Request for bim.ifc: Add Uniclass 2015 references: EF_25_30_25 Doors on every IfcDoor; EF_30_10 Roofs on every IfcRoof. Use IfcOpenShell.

First a look at what the model holds.

```python
import ifcopenshell

model = ifcopenshell.open("bim.ifc")
print(model.schema)
print("classifications:", [c.Name for c in model.by_type("IfcClassification")])
for ifc_class in ("IfcDoor", "IfcRoof", "IfcStair", "IfcWall", "IfcWindow"):
    print(ifc_class, len(model.by_type(ifc_class)))
```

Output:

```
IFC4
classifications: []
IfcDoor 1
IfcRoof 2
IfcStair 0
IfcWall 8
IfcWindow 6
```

```python
import ifcopenshell
import ifcopenshell.api.classification

model = ifcopenshell.open("bim.ifc")

system = ifcopenshell.api.classification.add_classification(model, classification="Uniclass 2015")

codes = {
    "IfcDoor": ("EF_25_30_25", "Doors"),
    "IfcRoof": ("EF_30_10", "Roofs"),
}
for ifc_class, (code, name) in codes.items():
    products = model.by_type(ifc_class)
    ifcopenshell.api.classification.add_reference(
        model, products=products, classification=system, identification=code, name=name
    )
    print(code, len(products))

model.write("bim_updated.ifc")
```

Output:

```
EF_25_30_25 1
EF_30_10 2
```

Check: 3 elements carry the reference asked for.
